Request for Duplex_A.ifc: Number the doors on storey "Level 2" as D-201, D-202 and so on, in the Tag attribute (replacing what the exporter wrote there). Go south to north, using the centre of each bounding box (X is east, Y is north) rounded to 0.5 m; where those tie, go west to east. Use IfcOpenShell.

First a look at what the model holds.

```python
import ifcopenshell
import ifcopenshell.util.element
import ifcopenshell.util.placement

model = ifcopenshell.open("Duplex_A.ifc")
print(model.schema)
storey = next(s for s in model.by_type("IfcBuildingStorey") if s.Name == "Level 2")
doors = [e for e in ifcopenshell.util.element.get_decomposition(storey) if e.is_a("IfcDoor")]
for e in sorted(doors, key=lambda e: e.id()):
    origin = ifcopenshell.util.placement.get_local_placement(e.ObjectPlacement)[:3, 3]
    print(e.id(), e.Tag, e.Name, origin.round(2) + 0.0, sep=" | ")
```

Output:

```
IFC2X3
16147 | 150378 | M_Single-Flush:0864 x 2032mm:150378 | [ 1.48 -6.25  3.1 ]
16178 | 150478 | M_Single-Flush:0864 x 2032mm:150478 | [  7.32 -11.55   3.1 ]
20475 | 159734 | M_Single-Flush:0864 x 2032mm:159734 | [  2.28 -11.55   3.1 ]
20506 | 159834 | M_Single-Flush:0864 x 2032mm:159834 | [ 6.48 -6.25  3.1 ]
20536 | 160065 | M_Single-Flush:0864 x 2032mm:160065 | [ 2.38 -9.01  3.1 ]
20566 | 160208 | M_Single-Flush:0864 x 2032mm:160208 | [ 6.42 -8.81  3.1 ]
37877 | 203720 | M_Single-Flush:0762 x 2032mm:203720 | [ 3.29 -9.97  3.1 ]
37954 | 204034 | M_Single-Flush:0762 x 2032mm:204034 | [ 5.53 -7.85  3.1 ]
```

```python
import ifcopenshell
import ifcopenshell.geom
import ifcopenshell.util.element
import ifcopenshell.util.shape

model = ifcopenshell.open("Duplex_A.ifc")
settings = ifcopenshell.geom.settings()
settings.set("use-world-coords", True)


def centre(element):
    shape = ifcopenshell.geom.create_shape(settings, element)
    return ifcopenshell.util.shape.get_bbox_centroid(shape.geometry)


storey = next(s for s in model.by_type("IfcBuildingStorey") if s.Name == "Level 2")
doors = [e for e in ifcopenshell.util.element.get_decomposition(storey) if e.is_a("IfcDoor")]

# Insertion points can sit at a corner or the storey origin, so sort by the geometry (in metres).
centres = {e: centre(e) for e in doors}
doors.sort(key=lambda e: (round(centres[e][1] / 0.5), centres[e][0]))

for i, e in enumerate(doors, start=1):
    number = f"D-2{i:02d}"
    e.Tag = number
    print(e.id(), number)

model.write("Duplex_A-out.ifc")
```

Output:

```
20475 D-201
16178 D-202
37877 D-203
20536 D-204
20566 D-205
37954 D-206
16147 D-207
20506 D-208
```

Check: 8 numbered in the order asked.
